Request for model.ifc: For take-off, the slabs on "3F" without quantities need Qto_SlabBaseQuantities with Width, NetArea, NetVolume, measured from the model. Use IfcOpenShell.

First a look at what the model holds.

```python
import ifcopenshell
import ifcopenshell.util.element
import ifcopenshell.util.unit

model = ifcopenshell.open("model.ifc")
print(model.schema)
for unit_type in ("LENGTHUNIT", "AREAUNIT", "VOLUMEUNIT"):
    print(unit_type, ifcopenshell.util.unit.calculate_unit_scale(model, unit_type))
storey = next(s for s in model.by_type("IfcBuildingStorey") if s.Name == "3F")
slabs = [e for e in ifcopenshell.util.element.get_decomposition(storey) if e.is_a("IfcSlab")]
for e in sorted(slabs, key=lambda e: e.id()):
    print(e.id(), e.is_a(), e.Name, list(ifcopenshell.util.element.get_psets(e, qtos_only=True)), sep=" | ")
```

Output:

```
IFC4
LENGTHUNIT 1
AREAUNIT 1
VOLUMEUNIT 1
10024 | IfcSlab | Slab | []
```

```python
import ifcopenshell
import ifcopenshell.api.pset
import ifcopenshell.geom
import ifcopenshell.util.element
import ifcopenshell.util.shape
import ifcopenshell.util.unit

model = ifcopenshell.open("model.ifc")
unit_scale = ifcopenshell.util.unit.calculate_unit_scale(model)
area_scale = ifcopenshell.util.unit.calculate_unit_scale(model, "AREAUNIT")
volume_scale = ifcopenshell.util.unit.calculate_unit_scale(model, "VOLUMEUNIT")
settings = ifcopenshell.geom.settings()

storey = next(s for s in model.by_type("IfcBuildingStorey") if s.Name == "3F")
slabs = [e for e in ifcopenshell.util.element.get_decomposition(storey) if e.is_a("IfcSlab")]

for e in sorted(slabs, key=lambda e: e.id()):
    if ifcopenshell.util.element.get_psets(e, qtos_only=True, should_inherit=False):
        continue
    # Geometry comes back in metres, in the element's own axes.
    shape = ifcopenshell.geom.create_shape(settings, e)
    values = {
        "Width": ifcopenshell.util.shape.get_z(shape.geometry) / unit_scale,
        "NetArea": ifcopenshell.util.shape.get_footprint_area(shape.geometry) / area_scale,
        "NetVolume": ifcopenshell.util.shape.get_volume(shape.geometry) / volume_scale,
    }
    qto = ifcopenshell.api.pset.add_qto(model, product=e, name="Qto_SlabBaseQuantities")
    ifcopenshell.api.pset.edit_qto(model, qto=qto, properties=values)
    print(e.id(), {k: round(v, 3) for k, v in values.items()})

model.write("model_rev.ifc")
```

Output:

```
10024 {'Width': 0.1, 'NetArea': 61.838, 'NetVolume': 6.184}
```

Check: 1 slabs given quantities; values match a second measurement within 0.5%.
